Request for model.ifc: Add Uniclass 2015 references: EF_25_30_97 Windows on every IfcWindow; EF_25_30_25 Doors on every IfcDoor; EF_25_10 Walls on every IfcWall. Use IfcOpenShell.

First a look at what the model holds.

```python
import ifcopenshell

model = ifcopenshell.open("model.ifc")
print(model.schema)
print("classifications:", [c.Name for c in model.by_type("IfcClassification")])
for ifc_class in ("IfcDoor", "IfcRoof", "IfcStair", "IfcWall", "IfcWindow"):
    print(ifc_class, len(model.by_type(ifc_class)))
```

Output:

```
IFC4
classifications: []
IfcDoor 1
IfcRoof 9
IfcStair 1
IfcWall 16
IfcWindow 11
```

```python
import ifcopenshell
import ifcopenshell.api.classification

model = ifcopenshell.open("model.ifc")

system = ifcopenshell.api.classification.add_classification(model, classification="Uniclass 2015")

codes = {
    "IfcWindow": ("EF_25_30_97", "Windows"),
    "IfcDoor": ("EF_25_30_25", "Doors"),
    "IfcWall": ("EF_25_10", "Walls"),
}
for ifc_class, (code, name) in codes.items():
    products = model.by_type(ifc_class)
    ifcopenshell.api.classification.add_reference(
        model, products=products, classification=system, identification=code, name=name
    )
    print(code, len(products))

model.write("model_edited.ifc")
```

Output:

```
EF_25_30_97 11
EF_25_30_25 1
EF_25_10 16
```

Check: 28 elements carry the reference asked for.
